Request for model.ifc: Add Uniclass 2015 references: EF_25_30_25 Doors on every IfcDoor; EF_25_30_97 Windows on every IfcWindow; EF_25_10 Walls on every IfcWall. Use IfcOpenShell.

First a look at what the model holds.

```python
import ifcopenshell

model = ifcopenshell.open("model.ifc")
print(model.schema)
print("classifications:", [c.Name for c in model.by_type("IfcClassification")])
for ifc_class in ("IfcDoor", "IfcRoof", "IfcStair", "IfcWall", "IfcWindow"):
    print(ifc_class, len(model.by_type(ifc_class)))
```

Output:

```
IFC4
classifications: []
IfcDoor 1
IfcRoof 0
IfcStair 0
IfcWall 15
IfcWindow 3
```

```python
import ifcopenshell
import ifcopenshell.api.classification

model = ifcopenshell.open("model.ifc")

system = ifcopenshell.api.classification.add_classification(model, classification="Uniclass 2015")

codes = {
    "IfcDoor": ("EF_25_30_25", "Doors"),
    "IfcWindow": ("EF_25_30_97", "Windows"),
    "IfcWall": ("EF_25_10", "Walls"),
}
for ifc_class, (code, name) in codes.items():
    products = model.by_type(ifc_class)
    ifcopenshell.api.classification.add_reference(
        model, products=products, classification=system, identification=code, name=name
    )
    print(code, len(products))

model.write("model-out.ifc")
```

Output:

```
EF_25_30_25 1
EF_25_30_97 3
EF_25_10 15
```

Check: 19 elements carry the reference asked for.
